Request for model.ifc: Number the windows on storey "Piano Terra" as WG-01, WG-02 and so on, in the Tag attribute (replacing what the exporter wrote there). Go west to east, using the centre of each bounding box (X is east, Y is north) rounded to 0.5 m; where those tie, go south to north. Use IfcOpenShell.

First a look at what the model holds.

```python
import ifcopenshell
import ifcopenshell.util.element
import ifcopenshell.util.placement

model = ifcopenshell.open("model.ifc")
print(model.schema)
storey = next(s for s in model.by_type("IfcBuildingStorey") if s.Name == "Piano Terra")
windows = [e for e in ifcopenshell.util.element.get_decomposition(storey) if e.is_a("IfcWindow")]
for e in sorted(windows, key=lambda e: e.id()):
    origin = ifcopenshell.util.placement.get_local_placement(e.ObjectPlacement)[:3, 3]
    print(e.id(), e.Tag, e.Name, origin.round(2) + 0.0, sep=" | ")
```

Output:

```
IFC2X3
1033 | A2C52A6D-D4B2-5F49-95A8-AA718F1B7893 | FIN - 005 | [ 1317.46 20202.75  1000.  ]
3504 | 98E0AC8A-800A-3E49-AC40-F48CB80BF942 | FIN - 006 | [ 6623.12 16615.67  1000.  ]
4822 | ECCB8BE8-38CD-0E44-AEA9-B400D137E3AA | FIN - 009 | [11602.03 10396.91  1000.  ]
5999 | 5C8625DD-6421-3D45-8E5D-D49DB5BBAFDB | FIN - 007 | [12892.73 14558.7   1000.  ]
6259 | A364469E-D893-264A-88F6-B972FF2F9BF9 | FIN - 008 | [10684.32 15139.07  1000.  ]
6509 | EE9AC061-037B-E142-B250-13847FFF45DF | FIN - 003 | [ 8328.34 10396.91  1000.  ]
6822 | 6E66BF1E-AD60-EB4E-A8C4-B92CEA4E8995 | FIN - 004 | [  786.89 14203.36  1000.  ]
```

```python
import ifcopenshell
import ifcopenshell.geom
import ifcopenshell.util.element
import ifcopenshell.util.shape

model = ifcopenshell.open("model.ifc")
settings = ifcopenshell.geom.settings()
settings.set("use-world-coords", True)


def centre(element):
    shape = ifcopenshell.geom.create_shape(settings, element)
    return ifcopenshell.util.shape.get_bbox_centroid(shape.geometry)


storey = next(s for s in model.by_type("IfcBuildingStorey") if s.Name == "Piano Terra")
windows = [e for e in ifcopenshell.util.element.get_decomposition(storey) if e.is_a("IfcWindow")]

# Insertion points can sit at a corner or the storey origin, so sort by the geometry (in metres).
centres = {e: centre(e) for e in windows}
windows.sort(key=lambda e: (round(centres[e][0] / 0.5), centres[e][1]))

for i, e in enumerate(windows, start=1):
    number = f"WG-{i:02d}"
    e.Tag = number
    print(e.id(), number)

model.write("model_updated.ifc")
```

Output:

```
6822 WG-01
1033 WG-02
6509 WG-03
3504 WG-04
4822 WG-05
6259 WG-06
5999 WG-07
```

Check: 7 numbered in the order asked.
